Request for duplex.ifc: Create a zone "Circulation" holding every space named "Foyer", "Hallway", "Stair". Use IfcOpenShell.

First a look at what the model holds.

```python
import ifcopenshell

model = ifcopenshell.open("duplex.ifc")
print(model.schema)
seen = {}
for space in model.by_type("IfcSpace"):
    seen[space.LongName] = seen.get(space.LongName, 0) + 1
for name, count in sorted(seen.items(), key=str):
    print(count, "x", name)
print("zones:", [z.Name for z in model.by_type("IfcZone")][:20])
```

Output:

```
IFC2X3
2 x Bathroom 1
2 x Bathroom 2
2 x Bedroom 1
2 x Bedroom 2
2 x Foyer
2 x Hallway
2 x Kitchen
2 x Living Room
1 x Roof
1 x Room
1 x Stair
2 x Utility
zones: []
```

```python
import ifcopenshell
import ifcopenshell.api.group
import ifcopenshell.api.root

model = ifcopenshell.open("duplex.ifc")

names = {"Foyer", "Hallway", "Stair"}
spaces = [s for s in model.by_type("IfcSpace") if s.LongName in names]

zone = ifcopenshell.api.root.create_entity(model, ifc_class="IfcZone", name="Circulation")
ifcopenshell.api.group.assign_group(model, products=spaces, group=zone)
print(len(spaces), "spaces in", zone.Name)

model.write("duplex_v2.ifc")
```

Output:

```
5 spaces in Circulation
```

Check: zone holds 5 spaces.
